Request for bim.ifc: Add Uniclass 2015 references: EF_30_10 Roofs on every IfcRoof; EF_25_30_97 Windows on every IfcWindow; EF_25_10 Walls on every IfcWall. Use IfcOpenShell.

First a look at what the model holds.

```python
import ifcopenshell

model = ifcopenshell.open("bim.ifc")
print(model.schema)
print("classifications:", [c.Name for c in model.by_type("IfcClassification")])
for ifc_class in ("IfcDoor", "IfcRoof", "IfcStair", "IfcWall", "IfcWindow"):
    print(ifc_class, len(model.by_type(ifc_class)))
```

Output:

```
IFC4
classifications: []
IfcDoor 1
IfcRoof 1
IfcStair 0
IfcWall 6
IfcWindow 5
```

```python
import ifcopenshell
import ifcopenshell.api.classification

model = ifcopenshell.open("bim.ifc")

system = ifcopenshell.api.classification.add_classification(model, classification="Uniclass 2015")

codes = {
    "IfcRoof": ("EF_30_10", "Roofs"),
    "IfcWindow": ("EF_25_30_97", "Windows"),
    "IfcWall": ("EF_25_10", "Walls"),
}
for ifc_class, (code, name) in codes.items():
    products = model.by_type(ifc_class)
    ifcopenshell.api.classification.add_reference(
        model, products=products, classification=system, identification=code, name=name
    )
    print(code, len(products))

model.write("bim-out.ifc")
```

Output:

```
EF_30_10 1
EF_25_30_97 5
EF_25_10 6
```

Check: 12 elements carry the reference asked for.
